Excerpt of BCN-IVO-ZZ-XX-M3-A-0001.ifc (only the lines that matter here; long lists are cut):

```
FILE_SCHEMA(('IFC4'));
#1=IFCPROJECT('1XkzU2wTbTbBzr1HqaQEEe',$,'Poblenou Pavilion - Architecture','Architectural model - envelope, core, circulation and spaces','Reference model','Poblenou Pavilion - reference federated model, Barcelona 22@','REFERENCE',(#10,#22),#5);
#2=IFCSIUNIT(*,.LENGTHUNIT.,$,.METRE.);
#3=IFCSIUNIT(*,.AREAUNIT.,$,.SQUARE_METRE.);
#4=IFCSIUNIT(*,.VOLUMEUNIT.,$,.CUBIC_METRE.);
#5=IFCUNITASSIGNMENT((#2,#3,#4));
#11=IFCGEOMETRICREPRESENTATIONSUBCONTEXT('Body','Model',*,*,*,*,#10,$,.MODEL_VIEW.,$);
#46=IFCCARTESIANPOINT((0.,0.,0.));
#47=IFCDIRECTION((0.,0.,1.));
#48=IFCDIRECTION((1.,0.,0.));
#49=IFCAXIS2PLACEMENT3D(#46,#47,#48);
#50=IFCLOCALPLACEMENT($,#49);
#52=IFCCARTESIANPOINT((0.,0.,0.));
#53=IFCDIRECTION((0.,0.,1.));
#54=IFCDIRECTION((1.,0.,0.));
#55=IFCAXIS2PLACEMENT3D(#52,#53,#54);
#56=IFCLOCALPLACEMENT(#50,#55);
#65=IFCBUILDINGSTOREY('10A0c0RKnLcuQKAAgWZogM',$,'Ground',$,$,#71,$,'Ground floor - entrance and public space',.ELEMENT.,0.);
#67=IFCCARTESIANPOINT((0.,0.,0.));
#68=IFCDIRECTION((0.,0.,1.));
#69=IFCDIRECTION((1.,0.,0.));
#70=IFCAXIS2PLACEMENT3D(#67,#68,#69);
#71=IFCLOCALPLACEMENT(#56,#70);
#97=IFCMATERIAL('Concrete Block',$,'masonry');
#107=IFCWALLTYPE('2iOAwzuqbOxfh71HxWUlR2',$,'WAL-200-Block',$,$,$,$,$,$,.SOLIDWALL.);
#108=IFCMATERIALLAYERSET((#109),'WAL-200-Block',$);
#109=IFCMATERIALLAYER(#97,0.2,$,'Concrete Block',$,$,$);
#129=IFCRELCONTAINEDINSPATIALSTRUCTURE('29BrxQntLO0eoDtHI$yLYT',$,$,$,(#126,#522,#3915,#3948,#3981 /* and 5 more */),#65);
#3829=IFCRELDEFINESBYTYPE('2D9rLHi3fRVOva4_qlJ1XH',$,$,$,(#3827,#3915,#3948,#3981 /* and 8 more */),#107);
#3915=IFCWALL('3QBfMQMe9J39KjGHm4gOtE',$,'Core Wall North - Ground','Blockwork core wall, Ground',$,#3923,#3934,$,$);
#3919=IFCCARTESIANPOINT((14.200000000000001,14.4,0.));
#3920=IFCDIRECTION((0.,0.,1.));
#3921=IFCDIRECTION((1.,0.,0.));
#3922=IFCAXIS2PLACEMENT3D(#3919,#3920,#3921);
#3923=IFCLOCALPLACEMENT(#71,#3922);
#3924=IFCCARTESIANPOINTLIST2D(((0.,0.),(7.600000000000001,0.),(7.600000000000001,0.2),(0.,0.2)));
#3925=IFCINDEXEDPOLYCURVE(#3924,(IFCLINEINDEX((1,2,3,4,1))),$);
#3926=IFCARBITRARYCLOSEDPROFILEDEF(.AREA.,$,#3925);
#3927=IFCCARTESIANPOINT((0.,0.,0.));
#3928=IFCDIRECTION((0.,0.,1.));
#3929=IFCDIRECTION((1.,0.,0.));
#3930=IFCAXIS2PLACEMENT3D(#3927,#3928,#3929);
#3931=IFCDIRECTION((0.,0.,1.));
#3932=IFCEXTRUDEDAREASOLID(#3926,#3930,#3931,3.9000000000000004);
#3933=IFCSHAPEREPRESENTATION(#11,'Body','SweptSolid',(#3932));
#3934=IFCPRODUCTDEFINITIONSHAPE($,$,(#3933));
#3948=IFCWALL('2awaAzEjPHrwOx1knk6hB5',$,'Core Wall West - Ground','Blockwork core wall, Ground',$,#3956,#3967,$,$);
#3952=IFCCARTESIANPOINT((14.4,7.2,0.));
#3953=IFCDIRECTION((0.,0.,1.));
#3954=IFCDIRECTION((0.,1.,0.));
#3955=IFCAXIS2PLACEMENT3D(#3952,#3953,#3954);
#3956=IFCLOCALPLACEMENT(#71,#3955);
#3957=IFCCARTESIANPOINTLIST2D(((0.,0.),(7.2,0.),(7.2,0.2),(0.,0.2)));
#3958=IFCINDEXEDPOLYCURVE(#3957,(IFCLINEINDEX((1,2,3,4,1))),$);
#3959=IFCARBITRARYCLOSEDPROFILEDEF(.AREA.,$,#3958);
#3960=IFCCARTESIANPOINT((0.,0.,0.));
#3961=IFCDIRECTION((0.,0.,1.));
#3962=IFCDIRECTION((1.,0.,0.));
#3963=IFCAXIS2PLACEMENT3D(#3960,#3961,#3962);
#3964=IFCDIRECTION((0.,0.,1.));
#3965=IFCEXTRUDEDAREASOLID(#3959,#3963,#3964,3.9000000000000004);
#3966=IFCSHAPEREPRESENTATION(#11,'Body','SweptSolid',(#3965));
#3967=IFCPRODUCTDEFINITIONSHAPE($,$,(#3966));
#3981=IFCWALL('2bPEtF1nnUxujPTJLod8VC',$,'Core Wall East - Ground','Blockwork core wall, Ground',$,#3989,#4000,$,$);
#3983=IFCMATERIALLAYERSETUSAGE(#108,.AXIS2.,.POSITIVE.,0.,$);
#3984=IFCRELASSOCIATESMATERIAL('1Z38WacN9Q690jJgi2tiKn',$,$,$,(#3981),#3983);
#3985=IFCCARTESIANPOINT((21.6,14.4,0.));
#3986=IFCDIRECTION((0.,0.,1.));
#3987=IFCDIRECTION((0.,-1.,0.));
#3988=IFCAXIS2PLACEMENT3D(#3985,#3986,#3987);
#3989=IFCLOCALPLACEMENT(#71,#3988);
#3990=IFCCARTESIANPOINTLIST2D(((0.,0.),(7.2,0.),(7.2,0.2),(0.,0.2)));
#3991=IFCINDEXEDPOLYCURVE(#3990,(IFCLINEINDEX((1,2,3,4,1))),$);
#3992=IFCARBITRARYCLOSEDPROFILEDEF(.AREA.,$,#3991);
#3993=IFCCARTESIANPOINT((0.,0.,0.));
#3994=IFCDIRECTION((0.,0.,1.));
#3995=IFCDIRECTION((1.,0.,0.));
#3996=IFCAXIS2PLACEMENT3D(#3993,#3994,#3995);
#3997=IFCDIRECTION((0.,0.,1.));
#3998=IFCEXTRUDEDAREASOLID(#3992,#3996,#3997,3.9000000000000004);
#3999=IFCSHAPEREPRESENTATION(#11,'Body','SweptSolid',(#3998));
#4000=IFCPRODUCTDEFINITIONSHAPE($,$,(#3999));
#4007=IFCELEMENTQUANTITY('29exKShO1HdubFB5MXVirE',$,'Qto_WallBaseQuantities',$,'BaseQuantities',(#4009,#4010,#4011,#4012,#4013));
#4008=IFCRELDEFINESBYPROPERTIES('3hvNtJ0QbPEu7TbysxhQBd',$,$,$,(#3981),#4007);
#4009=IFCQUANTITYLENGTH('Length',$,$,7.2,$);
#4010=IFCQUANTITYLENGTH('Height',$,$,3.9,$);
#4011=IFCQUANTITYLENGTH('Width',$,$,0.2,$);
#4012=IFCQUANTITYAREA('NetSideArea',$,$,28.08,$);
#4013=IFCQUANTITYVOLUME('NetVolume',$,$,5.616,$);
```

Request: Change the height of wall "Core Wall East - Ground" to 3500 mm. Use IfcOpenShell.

```python
import ifcopenshell
import ifcopenshell.api.pset
import ifcopenshell.geom
import ifcopenshell.util.element
import ifcopenshell.util.representation
import ifcopenshell.util.shape
import ifcopenshell.util.unit

model = ifcopenshell.open("BCN-IVO-ZZ-XX-M3-A-0001.ifc")
unit_scale = ifcopenshell.util.unit.calculate_unit_scale(model)
area_scale = ifcopenshell.util.unit.calculate_unit_scale(model, "AREAUNIT")
volume_scale = ifcopenshell.util.unit.calculate_unit_scale(model, "VOLUMEUNIT")
settings = ifcopenshell.geom.settings()


def volume(element):
    """Net volume in cubic metres, openings subtracted."""
    shape = ifcopenshell.geom.create_shape(settings, element)
    return ifcopenshell.util.shape.get_volume(shape.geometry)


wall = model.by_guid("2bPEtF1nnUxujPTJLod8VC")
before = volume(wall)

body = ifcopenshell.util.representation.get_representation(wall, "Model", "Body")
solid = body.Items[0]
old_height = solid.Depth
solid.Depth = 3.5 / unit_scale
after = volume(wall)
thickness = 0.2  # wall thickness in metres

# Update the stored height, areas and volumes.
qto = model.by_id(ifcopenshell.util.element.get_pset(wall, "Qto_WallBaseQuantities", should_inherit=False)["id"])
ifcopenshell.api.pset.edit_qto(model, qto=qto, properties={
    "Height": solid.Depth,
    "NetSideArea": after / thickness / area_scale,
    "NetVolume": after / volume_scale,
})

print(f"height {old_height:g} -> {solid.Depth:g}, volume {before:.3f} -> {after:.3f} m3")

model.write("BCN-IVO-ZZ-XX-M3-A-0001_rev.ifc")
```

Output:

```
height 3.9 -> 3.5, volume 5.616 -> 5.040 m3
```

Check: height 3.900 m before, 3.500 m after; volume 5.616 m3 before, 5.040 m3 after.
